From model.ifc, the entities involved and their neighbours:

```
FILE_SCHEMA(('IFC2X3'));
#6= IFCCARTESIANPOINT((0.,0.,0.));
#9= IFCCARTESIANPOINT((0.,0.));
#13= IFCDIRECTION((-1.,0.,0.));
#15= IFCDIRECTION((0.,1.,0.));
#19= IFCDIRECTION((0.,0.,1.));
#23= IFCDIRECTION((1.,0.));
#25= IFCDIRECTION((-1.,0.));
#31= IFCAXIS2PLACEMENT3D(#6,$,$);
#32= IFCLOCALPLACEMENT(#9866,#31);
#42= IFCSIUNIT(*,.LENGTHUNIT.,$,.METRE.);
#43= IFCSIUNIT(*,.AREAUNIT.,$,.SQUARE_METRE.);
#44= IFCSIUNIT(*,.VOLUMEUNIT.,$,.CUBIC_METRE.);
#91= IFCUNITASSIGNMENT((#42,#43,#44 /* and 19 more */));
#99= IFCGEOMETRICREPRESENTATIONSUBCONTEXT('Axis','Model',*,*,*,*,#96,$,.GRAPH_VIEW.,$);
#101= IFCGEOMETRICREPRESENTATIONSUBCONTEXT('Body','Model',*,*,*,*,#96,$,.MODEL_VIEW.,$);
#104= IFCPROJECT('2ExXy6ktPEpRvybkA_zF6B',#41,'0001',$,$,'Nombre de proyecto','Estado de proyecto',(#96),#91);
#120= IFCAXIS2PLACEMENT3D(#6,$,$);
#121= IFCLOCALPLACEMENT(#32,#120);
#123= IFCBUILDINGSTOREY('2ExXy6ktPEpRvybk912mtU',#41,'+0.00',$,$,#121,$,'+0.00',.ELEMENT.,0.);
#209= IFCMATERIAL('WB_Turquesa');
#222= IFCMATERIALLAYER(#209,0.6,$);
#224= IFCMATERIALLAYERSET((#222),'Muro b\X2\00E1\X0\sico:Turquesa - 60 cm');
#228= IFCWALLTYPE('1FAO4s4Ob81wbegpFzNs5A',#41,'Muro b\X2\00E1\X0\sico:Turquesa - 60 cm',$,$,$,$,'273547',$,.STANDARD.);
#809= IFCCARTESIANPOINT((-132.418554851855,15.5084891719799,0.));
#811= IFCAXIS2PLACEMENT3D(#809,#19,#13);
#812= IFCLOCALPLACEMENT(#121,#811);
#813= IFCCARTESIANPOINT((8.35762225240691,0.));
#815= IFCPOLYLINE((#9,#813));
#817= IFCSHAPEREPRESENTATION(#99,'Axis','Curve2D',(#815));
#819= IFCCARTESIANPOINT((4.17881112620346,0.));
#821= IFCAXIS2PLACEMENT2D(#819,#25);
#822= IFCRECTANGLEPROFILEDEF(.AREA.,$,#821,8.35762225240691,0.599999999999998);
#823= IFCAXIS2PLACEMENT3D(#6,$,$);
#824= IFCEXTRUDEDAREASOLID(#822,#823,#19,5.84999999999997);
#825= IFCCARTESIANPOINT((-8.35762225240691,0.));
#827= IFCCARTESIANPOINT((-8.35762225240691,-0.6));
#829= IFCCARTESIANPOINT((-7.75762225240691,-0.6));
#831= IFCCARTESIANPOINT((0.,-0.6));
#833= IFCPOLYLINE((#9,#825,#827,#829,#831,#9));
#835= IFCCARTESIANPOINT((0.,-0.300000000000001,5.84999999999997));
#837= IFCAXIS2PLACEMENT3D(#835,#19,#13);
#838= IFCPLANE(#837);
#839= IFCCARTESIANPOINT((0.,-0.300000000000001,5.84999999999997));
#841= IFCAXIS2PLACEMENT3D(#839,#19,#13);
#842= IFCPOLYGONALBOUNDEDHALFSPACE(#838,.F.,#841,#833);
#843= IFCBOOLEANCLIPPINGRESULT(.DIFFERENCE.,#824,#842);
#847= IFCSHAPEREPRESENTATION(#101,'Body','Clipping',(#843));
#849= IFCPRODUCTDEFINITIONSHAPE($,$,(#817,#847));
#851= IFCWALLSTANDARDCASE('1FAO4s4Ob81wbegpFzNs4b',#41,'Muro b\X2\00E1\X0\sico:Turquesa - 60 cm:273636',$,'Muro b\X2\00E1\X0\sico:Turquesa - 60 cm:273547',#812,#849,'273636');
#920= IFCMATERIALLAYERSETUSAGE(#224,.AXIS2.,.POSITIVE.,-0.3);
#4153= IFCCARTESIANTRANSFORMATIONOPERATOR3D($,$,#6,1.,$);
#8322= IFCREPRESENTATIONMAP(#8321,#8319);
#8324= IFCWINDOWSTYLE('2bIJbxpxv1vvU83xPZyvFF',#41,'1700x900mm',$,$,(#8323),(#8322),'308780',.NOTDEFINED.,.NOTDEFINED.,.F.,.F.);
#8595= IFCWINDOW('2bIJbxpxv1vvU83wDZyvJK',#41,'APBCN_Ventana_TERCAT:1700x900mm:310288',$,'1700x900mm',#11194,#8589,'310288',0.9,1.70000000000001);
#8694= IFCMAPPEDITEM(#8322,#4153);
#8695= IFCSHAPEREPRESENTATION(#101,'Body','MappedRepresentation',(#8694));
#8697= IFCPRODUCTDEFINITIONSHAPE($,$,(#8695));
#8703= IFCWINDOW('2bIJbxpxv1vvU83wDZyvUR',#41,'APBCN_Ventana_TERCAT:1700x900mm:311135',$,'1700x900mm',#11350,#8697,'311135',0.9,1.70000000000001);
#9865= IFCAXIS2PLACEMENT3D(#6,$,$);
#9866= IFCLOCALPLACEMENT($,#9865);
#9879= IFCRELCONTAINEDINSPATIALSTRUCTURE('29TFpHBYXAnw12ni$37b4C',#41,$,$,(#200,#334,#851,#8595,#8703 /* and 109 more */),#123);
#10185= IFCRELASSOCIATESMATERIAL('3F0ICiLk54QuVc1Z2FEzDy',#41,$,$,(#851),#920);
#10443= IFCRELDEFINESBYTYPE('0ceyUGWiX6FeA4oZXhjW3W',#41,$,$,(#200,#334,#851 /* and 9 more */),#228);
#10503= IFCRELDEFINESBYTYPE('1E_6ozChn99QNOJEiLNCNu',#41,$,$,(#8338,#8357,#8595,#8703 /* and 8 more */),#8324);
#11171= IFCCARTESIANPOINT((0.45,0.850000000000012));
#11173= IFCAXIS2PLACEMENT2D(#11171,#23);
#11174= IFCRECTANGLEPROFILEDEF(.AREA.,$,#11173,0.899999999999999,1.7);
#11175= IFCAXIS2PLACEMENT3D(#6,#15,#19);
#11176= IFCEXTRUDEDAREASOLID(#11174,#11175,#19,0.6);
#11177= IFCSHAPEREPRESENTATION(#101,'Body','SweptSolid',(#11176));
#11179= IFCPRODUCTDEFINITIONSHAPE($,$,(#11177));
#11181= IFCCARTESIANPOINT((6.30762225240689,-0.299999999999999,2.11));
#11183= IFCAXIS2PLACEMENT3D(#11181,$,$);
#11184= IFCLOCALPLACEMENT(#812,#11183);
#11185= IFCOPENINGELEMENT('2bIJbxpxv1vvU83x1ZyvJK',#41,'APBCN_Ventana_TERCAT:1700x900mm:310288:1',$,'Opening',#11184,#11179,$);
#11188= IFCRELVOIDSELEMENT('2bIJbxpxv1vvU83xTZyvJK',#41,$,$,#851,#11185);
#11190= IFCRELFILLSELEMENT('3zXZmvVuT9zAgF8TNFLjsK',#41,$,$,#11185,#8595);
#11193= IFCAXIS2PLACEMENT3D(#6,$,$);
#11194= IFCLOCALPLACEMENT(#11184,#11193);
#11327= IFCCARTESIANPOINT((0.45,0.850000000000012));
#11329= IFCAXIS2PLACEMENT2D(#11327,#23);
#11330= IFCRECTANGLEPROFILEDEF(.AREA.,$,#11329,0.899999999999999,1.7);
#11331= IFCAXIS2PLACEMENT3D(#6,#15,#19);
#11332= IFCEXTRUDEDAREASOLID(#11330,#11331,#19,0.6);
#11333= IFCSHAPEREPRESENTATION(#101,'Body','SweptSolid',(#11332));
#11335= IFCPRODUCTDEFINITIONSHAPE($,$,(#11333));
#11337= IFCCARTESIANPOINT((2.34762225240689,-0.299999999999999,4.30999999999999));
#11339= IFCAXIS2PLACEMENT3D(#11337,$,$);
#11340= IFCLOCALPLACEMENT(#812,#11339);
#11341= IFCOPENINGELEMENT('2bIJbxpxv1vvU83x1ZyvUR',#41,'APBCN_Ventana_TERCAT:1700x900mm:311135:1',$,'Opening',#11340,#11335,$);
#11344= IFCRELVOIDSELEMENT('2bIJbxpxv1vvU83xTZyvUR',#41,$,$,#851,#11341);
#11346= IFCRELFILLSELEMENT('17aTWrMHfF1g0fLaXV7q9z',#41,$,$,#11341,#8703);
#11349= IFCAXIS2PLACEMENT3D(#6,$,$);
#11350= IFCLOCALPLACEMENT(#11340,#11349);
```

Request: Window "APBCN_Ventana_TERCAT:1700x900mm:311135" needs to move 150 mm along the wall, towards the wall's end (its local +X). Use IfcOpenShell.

```python
import ifcopenshell
import ifcopenshell.api.geometry
import ifcopenshell.util.placement
import ifcopenshell.util.unit

model = ifcopenshell.open("model.ifc")
unit_scale = ifcopenshell.util.unit.calculate_unit_scale(model)

window = model.by_guid("2bIJbxpxv1vvU83wDZyvUR")
opening = window.FillsVoids[0].RelatingOpeningElement
wall = opening.VoidsElements[0].RelatingBuildingElement

wall_matrix = ifcopenshell.util.placement.get_local_placement(wall.ObjectPlacement)
shift = wall_matrix[:3, 0] * 0.15 / unit_scale
before = ifcopenshell.util.placement.get_local_placement(window.ObjectPlacement)[:3, 3].copy()

# The window is placed relative to its opening, so it follows when the opening moves.
matrix = ifcopenshell.util.placement.get_local_placement(opening.ObjectPlacement)
matrix[:3, 3] += shift
ifcopenshell.api.geometry.edit_object_placement(
    model, product=opening, matrix=matrix, is_si=False, should_transform_children=True
)

after = ifcopenshell.util.placement.get_local_placement(window.ObjectPlacement)[:3, 3]
print("window moved by", (after - before).round(3) + 0.0)

model.write("model_rev.ifc")
```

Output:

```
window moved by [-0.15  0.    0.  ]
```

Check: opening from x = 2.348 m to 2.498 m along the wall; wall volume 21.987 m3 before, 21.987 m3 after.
